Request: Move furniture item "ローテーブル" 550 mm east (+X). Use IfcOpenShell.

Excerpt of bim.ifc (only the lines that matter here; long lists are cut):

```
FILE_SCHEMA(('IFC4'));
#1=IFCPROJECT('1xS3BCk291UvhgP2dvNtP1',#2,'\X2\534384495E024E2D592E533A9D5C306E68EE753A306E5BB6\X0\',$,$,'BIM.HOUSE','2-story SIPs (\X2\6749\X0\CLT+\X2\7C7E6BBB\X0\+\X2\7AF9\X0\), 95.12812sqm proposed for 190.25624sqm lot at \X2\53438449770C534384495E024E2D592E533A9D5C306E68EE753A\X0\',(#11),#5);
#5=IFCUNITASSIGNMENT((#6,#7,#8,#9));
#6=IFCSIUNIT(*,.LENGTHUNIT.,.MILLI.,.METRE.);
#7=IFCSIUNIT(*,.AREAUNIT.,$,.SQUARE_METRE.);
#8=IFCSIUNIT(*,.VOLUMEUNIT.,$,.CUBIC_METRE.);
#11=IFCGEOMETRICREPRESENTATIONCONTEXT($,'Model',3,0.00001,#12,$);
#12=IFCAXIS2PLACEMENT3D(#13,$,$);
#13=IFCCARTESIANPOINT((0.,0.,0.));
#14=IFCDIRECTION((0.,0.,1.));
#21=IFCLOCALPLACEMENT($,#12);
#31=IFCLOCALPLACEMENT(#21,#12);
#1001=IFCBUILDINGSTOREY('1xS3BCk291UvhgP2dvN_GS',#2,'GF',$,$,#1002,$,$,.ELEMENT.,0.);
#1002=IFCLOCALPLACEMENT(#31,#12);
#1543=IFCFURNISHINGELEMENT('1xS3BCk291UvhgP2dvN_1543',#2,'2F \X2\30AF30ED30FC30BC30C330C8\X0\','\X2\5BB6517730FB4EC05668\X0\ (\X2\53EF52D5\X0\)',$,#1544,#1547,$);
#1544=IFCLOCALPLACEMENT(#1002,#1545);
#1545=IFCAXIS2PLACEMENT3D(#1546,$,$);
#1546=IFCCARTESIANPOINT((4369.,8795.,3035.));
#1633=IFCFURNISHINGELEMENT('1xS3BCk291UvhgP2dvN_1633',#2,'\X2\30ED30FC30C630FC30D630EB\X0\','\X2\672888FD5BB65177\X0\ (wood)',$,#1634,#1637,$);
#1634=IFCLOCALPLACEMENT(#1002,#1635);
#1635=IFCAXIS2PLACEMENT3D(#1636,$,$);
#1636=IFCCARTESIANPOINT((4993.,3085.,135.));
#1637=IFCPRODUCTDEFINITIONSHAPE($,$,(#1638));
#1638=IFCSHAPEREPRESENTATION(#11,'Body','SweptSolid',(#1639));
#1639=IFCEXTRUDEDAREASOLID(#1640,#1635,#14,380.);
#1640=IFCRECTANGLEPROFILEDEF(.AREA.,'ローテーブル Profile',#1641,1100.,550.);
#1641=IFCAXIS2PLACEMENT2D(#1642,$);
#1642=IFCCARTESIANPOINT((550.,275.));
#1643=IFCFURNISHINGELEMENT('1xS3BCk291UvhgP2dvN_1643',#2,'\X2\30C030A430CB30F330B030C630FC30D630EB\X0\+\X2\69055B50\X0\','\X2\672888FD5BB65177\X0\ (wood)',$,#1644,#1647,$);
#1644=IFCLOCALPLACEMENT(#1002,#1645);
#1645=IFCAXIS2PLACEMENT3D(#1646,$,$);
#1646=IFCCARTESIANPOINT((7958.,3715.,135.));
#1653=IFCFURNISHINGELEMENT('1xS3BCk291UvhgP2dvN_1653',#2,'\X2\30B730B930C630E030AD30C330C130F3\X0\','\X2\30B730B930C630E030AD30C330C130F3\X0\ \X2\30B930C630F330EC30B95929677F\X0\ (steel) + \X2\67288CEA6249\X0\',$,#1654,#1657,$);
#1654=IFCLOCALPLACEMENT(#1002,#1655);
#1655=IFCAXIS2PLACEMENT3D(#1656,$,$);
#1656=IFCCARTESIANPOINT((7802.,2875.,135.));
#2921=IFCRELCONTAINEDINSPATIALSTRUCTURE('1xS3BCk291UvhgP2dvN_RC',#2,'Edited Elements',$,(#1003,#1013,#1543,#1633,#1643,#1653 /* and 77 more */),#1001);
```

```python
import ifcopenshell
import ifcopenshell.api.geometry
import ifcopenshell.util.placement
import ifcopenshell.util.unit

model = ifcopenshell.open("bim.ifc")
unit_scale = ifcopenshell.util.unit.calculate_unit_scale(model)

item = model.by_guid("1xS3BCk291UvhgP2dvN_1633")
matrix = ifcopenshell.util.placement.get_local_placement(item.ObjectPlacement)
matrix[0, 3] += 0.55 / unit_scale
ifcopenshell.api.geometry.edit_object_placement(model, product=item, matrix=matrix, is_si=False)

print(ifcopenshell.util.placement.get_local_placement(item.ObjectPlacement).round(3) + 0.0)

model.write("bim_edited.ifc")
```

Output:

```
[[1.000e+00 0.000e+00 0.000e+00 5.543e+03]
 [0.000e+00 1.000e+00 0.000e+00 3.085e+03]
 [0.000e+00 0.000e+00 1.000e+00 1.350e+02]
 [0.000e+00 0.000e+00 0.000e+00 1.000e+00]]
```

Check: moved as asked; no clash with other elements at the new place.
